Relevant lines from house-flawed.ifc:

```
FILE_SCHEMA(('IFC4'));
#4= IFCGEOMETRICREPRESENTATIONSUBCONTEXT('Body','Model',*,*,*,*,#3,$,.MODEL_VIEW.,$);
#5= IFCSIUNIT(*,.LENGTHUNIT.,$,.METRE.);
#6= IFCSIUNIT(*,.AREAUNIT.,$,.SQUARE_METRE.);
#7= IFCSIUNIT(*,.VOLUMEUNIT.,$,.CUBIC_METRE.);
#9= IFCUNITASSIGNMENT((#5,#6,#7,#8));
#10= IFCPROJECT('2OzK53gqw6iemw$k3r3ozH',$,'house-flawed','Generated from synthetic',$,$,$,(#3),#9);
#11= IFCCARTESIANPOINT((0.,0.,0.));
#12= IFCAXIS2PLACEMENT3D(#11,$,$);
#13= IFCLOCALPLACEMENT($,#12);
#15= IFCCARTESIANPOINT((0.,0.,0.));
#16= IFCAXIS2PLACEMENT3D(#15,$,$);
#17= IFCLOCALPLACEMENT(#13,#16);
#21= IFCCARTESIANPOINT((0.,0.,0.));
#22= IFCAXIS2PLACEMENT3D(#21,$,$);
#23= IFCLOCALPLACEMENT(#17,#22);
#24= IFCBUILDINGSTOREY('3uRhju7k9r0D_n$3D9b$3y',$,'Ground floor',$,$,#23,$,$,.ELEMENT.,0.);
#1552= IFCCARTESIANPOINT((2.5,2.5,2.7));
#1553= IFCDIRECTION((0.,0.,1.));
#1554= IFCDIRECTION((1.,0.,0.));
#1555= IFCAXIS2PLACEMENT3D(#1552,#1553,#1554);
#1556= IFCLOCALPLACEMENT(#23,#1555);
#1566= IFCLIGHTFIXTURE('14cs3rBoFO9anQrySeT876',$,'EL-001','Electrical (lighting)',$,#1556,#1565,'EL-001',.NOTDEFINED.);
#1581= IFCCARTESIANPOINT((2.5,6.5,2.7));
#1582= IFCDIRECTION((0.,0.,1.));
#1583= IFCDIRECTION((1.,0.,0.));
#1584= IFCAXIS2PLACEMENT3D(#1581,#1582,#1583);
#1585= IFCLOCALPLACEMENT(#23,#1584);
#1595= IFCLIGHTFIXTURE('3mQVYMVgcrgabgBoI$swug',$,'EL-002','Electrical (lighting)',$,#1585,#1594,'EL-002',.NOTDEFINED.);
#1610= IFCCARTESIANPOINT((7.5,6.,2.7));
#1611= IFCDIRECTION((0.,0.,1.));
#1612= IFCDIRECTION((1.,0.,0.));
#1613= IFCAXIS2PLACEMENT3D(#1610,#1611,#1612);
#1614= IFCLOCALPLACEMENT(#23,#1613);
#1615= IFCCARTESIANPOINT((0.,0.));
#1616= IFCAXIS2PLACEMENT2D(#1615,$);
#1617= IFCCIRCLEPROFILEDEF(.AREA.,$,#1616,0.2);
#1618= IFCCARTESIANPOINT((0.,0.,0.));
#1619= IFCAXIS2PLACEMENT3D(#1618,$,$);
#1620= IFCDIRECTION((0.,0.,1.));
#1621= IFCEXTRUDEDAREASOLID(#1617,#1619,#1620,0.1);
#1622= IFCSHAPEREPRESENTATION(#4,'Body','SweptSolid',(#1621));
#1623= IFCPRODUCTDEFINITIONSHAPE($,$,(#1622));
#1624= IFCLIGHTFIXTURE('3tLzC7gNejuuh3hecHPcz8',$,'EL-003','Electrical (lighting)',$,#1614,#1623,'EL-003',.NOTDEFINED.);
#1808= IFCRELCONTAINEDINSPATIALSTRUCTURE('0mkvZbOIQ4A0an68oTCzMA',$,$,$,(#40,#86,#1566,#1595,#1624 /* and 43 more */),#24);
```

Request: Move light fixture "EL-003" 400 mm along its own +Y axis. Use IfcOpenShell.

```python
import ifcopenshell
import ifcopenshell.api.geometry
import ifcopenshell.util.placement
import ifcopenshell.util.unit

model = ifcopenshell.open("house-flawed.ifc")
unit_scale = ifcopenshell.util.unit.calculate_unit_scale(model)

item = model.by_id(1624)
matrix = ifcopenshell.util.placement.get_local_placement(item.ObjectPlacement)
matrix[:3, 3] += matrix[:3, 1] * 0.4 / unit_scale
ifcopenshell.api.geometry.edit_object_placement(model, product=item, matrix=matrix, is_si=False)

print(ifcopenshell.util.placement.get_local_placement(item.ObjectPlacement).round(3) + 0.0)

model.write("house-flawed_rev.ifc")
```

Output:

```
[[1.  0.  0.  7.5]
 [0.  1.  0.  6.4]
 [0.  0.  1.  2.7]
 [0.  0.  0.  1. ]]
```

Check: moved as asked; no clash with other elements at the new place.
